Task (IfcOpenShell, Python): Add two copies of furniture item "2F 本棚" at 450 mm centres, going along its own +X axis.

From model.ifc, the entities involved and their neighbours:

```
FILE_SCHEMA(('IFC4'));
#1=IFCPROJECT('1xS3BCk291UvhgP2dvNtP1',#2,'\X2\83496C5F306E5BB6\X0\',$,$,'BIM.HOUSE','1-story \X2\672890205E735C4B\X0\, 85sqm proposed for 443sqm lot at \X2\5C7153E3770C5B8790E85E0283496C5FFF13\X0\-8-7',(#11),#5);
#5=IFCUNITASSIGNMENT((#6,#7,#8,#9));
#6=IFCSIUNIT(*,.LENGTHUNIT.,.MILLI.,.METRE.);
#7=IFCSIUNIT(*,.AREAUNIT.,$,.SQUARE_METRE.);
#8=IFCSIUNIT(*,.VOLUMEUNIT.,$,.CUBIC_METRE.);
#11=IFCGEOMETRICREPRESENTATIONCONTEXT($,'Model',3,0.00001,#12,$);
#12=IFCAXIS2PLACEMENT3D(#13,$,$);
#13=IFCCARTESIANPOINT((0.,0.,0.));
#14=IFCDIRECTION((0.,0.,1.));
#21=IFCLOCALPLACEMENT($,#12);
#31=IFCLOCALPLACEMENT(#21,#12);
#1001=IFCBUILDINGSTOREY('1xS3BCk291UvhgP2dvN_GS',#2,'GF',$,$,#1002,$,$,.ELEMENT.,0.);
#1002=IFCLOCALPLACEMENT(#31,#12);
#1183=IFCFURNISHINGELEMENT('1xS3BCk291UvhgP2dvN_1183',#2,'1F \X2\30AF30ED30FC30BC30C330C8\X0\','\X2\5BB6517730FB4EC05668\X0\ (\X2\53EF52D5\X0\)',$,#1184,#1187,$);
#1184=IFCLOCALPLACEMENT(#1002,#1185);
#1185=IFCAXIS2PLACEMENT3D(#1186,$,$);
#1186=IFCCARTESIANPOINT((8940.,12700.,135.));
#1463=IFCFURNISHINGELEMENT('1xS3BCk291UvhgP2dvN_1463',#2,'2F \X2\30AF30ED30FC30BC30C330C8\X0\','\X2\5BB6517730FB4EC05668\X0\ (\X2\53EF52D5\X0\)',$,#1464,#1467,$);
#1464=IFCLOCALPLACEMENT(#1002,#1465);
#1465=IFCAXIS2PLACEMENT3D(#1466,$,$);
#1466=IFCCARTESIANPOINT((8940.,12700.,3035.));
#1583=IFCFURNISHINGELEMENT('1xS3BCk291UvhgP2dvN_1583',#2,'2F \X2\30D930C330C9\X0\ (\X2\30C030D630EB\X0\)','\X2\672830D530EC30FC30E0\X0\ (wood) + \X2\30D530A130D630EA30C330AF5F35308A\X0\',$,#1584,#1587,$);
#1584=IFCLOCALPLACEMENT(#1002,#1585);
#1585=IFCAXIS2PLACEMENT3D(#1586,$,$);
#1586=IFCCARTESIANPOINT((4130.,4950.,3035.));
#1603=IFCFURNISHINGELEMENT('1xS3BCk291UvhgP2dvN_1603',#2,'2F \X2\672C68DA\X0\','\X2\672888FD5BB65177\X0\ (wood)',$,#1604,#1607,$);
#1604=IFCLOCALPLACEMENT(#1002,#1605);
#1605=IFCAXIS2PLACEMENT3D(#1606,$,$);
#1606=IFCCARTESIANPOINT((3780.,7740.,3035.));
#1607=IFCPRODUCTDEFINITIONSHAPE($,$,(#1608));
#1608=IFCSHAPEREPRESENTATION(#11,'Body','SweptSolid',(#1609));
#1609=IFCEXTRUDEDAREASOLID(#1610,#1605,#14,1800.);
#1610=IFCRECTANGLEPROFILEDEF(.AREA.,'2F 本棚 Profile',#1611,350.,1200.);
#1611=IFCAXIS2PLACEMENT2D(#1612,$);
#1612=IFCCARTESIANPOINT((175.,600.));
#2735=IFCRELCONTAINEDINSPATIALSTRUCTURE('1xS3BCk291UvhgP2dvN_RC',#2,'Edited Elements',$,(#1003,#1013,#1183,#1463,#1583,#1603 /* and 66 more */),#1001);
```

```python
import ifcopenshell
import ifcopenshell.api.geometry
import ifcopenshell.api.root
import ifcopenshell.util.element
import ifcopenshell.util.placement

model = ifcopenshell.open("model.ifc")


def reuse_history(source, copy):
    """copy_class also copies each property set's owner history, people and application; keep the originals."""
    for rel in copy.IsDefinedBy:
        if rel.is_a("IfcRelDefinesByProperties") and (history := rel.RelatingPropertyDefinition.OwnerHistory):
            rel.RelatingPropertyDefinition.OwnerHistory = source.OwnerHistory
            ifcopenshell.util.element.remove_deep2(model, history)


source = model.by_guid("1xS3BCk291UvhgP2dvN_1603")
base = ifcopenshell.util.placement.get_local_placement(source.ObjectPlacement)
step = base[:3, 0] * 450.0

for i in range(1, 3):
    copy = ifcopenshell.api.root.copy_class(model, product=source)
    copy.Representation = ifcopenshell.util.element.copy_deep(
        model, source.Representation, exclude=["IfcGeometricRepresentationContext", "IfcRepresentationMap"]
    )
    reuse_history(source, copy)
    matrix = base.copy()
    matrix[:3, 3] += i * step
    print("added at", matrix[:3, 3].round(3) + 0.0)
    ifcopenshell.api.geometry.edit_object_placement(model, product=copy, matrix=matrix, is_si=False)

model.write("model_rev.ifc")
```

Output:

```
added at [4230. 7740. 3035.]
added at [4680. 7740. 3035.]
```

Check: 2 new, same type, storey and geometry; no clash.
